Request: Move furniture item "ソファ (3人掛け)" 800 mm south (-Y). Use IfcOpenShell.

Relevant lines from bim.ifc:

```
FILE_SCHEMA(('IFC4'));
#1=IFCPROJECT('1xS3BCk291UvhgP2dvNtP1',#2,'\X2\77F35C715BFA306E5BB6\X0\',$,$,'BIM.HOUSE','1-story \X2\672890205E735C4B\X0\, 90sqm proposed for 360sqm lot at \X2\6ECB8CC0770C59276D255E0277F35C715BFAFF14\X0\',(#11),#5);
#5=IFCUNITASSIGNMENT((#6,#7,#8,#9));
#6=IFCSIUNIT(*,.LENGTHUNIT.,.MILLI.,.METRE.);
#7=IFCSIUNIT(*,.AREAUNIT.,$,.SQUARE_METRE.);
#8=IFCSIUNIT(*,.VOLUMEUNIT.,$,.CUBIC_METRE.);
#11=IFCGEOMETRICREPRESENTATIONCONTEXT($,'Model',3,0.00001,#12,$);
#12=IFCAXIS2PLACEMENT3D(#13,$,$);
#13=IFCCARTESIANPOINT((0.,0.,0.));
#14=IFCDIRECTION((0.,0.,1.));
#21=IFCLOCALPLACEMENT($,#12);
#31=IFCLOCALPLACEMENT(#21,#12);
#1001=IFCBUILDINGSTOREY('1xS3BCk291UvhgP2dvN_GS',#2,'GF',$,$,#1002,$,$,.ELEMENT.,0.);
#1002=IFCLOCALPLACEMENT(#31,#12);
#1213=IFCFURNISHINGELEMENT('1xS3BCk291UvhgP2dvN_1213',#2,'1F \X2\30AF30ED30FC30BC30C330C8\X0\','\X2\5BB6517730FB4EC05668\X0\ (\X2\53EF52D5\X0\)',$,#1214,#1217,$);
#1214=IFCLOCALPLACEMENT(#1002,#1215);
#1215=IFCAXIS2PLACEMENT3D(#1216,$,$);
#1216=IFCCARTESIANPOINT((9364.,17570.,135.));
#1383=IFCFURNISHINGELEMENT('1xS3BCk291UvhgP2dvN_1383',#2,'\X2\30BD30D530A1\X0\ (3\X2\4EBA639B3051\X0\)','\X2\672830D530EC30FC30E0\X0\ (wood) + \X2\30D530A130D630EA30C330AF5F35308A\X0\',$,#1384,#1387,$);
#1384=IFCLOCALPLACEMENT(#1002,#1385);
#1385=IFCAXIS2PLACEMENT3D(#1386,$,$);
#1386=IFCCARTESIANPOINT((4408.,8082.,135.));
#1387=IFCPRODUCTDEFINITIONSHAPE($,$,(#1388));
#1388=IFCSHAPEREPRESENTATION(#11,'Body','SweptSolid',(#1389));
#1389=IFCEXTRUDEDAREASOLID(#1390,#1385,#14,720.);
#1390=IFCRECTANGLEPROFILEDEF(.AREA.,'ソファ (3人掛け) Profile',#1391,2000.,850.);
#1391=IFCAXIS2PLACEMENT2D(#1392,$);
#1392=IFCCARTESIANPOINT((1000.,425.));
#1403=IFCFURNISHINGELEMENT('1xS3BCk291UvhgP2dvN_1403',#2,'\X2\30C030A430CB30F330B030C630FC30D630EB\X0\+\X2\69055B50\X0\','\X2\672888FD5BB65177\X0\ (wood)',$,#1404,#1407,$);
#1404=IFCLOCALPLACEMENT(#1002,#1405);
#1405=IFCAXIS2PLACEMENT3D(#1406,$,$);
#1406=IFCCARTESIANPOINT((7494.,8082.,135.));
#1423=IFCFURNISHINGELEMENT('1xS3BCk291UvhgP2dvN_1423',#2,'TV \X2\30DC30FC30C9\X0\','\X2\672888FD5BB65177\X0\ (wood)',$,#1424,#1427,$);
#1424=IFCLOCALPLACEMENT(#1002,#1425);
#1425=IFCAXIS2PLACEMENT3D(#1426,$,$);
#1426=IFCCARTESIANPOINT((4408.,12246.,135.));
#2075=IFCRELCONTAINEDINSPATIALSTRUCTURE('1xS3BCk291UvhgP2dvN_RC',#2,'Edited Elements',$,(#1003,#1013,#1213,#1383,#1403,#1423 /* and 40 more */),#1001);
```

```python
import ifcopenshell
import ifcopenshell.api.geometry
import ifcopenshell.util.placement
import ifcopenshell.util.unit

model = ifcopenshell.open("bim.ifc")
unit_scale = ifcopenshell.util.unit.calculate_unit_scale(model)

item = model.by_id(1383)
matrix = ifcopenshell.util.placement.get_local_placement(item.ObjectPlacement)
matrix[1, 3] -= 0.8 / unit_scale
ifcopenshell.api.geometry.edit_object_placement(model, product=item, matrix=matrix, is_si=False)

print(ifcopenshell.util.placement.get_local_placement(item.ObjectPlacement).round(3) + 0.0)

model.write("bim_edited.ifc")
```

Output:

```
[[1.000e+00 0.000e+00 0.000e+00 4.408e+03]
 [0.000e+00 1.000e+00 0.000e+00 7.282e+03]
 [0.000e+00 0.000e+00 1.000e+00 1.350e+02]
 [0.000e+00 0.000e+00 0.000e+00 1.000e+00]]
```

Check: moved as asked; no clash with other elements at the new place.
